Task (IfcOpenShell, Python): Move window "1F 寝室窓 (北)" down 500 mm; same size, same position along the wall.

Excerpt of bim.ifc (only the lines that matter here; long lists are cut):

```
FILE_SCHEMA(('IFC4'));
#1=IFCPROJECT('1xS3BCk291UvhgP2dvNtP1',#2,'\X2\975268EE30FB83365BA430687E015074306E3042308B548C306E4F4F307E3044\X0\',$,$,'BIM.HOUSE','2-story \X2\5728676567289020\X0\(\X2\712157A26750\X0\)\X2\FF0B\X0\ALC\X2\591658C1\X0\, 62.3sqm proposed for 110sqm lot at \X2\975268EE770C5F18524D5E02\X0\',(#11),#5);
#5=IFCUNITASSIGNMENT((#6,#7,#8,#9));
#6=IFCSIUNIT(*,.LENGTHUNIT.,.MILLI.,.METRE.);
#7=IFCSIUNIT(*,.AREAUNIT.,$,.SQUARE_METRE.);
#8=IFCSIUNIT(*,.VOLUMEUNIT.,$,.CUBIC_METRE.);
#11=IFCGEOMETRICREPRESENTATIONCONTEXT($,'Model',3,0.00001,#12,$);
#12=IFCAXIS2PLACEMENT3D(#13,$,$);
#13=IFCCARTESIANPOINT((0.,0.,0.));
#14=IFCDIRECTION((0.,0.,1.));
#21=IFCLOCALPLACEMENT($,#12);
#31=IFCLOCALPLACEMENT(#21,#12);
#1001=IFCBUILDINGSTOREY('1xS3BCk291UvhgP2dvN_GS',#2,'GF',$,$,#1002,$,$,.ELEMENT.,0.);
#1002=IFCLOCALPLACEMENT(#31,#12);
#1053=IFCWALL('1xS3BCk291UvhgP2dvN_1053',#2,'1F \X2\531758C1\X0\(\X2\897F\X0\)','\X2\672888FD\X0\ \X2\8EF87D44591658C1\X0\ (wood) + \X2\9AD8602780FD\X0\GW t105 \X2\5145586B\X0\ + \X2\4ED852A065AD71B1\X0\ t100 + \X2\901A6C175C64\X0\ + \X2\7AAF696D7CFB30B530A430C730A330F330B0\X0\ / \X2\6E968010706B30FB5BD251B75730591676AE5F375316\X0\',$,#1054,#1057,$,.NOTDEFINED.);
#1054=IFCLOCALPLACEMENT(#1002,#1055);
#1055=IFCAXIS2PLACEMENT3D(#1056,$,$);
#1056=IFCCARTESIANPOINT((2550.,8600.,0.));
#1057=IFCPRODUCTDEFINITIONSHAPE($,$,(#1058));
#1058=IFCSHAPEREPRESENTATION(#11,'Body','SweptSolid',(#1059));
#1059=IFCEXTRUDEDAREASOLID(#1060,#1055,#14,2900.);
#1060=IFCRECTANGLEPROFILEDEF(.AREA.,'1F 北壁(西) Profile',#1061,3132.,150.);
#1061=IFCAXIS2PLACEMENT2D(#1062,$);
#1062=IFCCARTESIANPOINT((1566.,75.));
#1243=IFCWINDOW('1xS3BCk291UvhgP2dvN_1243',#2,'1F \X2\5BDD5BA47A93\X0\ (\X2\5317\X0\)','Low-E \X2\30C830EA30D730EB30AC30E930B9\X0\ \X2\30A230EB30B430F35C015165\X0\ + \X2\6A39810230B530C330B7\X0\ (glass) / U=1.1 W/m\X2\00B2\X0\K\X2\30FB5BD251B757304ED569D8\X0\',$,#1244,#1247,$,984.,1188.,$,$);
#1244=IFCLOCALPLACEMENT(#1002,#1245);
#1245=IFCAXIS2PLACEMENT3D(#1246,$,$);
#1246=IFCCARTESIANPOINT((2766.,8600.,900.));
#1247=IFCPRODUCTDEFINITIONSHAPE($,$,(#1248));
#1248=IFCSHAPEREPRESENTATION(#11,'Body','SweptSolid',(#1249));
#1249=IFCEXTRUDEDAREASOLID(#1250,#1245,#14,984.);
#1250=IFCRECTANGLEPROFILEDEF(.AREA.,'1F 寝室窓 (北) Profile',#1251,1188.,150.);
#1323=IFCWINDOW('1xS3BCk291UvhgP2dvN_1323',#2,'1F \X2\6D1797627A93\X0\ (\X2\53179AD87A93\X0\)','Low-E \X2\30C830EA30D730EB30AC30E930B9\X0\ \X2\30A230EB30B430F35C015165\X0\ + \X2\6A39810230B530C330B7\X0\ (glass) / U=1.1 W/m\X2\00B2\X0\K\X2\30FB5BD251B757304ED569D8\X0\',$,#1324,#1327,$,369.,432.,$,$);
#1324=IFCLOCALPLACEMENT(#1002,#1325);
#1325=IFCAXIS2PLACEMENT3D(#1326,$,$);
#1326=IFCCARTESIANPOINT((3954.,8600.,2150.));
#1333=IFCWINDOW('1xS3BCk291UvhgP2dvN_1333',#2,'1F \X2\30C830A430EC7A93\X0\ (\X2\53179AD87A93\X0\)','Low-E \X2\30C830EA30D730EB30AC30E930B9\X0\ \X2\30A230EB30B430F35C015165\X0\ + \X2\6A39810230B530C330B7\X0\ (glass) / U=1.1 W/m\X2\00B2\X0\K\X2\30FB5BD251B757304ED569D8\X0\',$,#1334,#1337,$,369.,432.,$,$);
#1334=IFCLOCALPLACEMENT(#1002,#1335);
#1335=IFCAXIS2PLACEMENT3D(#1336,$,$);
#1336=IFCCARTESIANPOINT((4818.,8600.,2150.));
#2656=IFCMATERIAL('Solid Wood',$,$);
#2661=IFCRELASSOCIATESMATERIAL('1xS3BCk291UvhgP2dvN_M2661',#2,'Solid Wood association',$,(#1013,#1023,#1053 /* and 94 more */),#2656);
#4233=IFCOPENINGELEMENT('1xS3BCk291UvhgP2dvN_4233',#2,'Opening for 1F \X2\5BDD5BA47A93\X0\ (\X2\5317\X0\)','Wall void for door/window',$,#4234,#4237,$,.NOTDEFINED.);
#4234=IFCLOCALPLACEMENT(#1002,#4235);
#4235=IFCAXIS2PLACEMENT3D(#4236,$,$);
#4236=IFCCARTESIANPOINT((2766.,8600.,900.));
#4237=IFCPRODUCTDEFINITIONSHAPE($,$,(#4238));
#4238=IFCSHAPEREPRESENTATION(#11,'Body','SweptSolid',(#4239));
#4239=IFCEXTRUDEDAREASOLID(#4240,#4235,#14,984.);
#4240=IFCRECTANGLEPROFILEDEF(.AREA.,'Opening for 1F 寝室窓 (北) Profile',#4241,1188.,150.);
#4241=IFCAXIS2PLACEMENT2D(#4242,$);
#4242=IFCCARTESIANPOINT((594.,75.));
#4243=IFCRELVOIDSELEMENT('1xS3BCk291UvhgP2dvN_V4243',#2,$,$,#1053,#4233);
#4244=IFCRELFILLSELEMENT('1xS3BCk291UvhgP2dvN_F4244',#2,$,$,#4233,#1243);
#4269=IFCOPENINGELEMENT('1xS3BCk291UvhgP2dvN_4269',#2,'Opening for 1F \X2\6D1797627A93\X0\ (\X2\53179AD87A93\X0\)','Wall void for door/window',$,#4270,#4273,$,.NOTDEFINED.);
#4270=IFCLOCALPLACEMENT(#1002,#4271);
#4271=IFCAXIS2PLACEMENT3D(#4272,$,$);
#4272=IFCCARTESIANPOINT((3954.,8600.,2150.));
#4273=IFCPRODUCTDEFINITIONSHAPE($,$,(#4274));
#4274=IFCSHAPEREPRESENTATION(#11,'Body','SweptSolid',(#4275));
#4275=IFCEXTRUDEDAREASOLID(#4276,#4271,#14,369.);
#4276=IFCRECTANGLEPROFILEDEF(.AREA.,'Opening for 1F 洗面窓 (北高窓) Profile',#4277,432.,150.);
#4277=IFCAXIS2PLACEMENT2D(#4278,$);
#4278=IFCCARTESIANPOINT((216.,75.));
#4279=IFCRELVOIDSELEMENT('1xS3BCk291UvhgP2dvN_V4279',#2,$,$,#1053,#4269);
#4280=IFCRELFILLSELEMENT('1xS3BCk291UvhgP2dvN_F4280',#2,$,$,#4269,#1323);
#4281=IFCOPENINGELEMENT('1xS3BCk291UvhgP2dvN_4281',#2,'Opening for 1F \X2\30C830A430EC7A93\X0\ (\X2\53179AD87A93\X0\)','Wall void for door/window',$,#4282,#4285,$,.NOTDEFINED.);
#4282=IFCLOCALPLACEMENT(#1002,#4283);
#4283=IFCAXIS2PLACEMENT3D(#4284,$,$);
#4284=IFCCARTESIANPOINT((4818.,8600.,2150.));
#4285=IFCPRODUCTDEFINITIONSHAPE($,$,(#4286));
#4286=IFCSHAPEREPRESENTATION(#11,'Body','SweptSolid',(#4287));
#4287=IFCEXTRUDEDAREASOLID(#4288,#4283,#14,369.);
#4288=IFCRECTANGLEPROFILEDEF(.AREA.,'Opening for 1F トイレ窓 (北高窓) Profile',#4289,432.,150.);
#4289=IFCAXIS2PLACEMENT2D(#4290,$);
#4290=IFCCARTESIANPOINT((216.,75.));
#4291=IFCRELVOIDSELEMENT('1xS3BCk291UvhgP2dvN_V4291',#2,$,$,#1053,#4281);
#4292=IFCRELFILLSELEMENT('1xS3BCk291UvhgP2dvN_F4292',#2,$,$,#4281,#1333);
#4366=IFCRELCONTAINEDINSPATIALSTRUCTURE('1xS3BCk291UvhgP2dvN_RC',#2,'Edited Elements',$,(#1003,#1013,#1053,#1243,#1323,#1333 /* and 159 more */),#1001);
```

```python
import numpy as np
import ifcopenshell
import ifcopenshell.api.geometry
import ifcopenshell.util.placement
import ifcopenshell.util.unit

model = ifcopenshell.open("bim.ifc")
unit_scale = ifcopenshell.util.unit.calculate_unit_scale(model)

window = model.by_guid("1xS3BCk291UvhgP2dvN_1243")
opening = window.FillsVoids[0].RelatingOpeningElement
dz = -0.5 / unit_scale

shift = np.array([0.0, 0.0, dz])
# The window is not placed relative to its opening, so move both.
for product in (opening, window):
    matrix = ifcopenshell.util.placement.get_local_placement(product.ObjectPlacement)
    matrix[:3, 3] += shift
    ifcopenshell.api.geometry.edit_object_placement(model, product=product, matrix=matrix, is_si=False)

print(f"moved by {dz * unit_scale:+.3f} m")

model.write("bim-out.ifc")
```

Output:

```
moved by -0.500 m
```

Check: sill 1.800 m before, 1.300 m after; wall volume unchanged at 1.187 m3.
